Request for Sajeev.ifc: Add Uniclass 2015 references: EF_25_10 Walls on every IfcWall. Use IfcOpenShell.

First a look at what the model holds.

```python
import ifcopenshell

model = ifcopenshell.open("Sajeev.ifc")
print(model.schema)
print("classifications:", [c.Name for c in model.by_type("IfcClassification")])
for ifc_class in ("IfcDoor", "IfcRoof", "IfcStair", "IfcWall", "IfcWindow"):
    print(ifc_class, len(model.by_type(ifc_class)))
```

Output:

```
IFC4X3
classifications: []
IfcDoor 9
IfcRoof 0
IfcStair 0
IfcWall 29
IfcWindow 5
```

```python
import ifcopenshell
import ifcopenshell.api.classification

model = ifcopenshell.open("Sajeev.ifc")

system = ifcopenshell.api.classification.add_classification(model, classification="Uniclass 2015")

codes = {
    "IfcWall": ("EF_25_10", "Walls"),
}
for ifc_class, (code, name) in codes.items():
    products = model.by_type(ifc_class)
    ifcopenshell.api.classification.add_reference(
        model, products=products, classification=system, identification=code, name=name
    )
    print(code, len(products))

model.write("Sajeev-out.ifc")
```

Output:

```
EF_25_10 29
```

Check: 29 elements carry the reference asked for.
